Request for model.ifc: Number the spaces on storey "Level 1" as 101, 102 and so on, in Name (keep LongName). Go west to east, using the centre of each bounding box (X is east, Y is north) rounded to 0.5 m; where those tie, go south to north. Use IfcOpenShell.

First a look at what the model holds.

```python
import ifcopenshell
import ifcopenshell.util.element
import ifcopenshell.util.placement

model = ifcopenshell.open("model.ifc")
print(model.schema)
storey = next(s for s in model.by_type("IfcBuildingStorey") if s.Name == "Level 1")
spaces = [e for e in ifcopenshell.util.element.get_decomposition(storey) if e.is_a("IfcSpace")]
for e in sorted(spaces, key=lambda e: e.id()):
    origin = ifcopenshell.util.placement.get_local_placement(e.ObjectPlacement)[:3, 3]
    print(e.id(), e.Name, e.LongName, origin.round(2) + 0.0, sep=" | ")
```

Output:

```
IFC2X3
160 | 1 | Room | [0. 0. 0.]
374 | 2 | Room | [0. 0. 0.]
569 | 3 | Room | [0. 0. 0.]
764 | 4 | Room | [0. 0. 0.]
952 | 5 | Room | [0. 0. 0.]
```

```python
import ifcopenshell
import ifcopenshell.geom
import ifcopenshell.util.element
import ifcopenshell.util.shape

model = ifcopenshell.open("model.ifc")
settings = ifcopenshell.geom.settings()
settings.set("use-world-coords", True)


def centre(element):
    shape = ifcopenshell.geom.create_shape(settings, element)
    return ifcopenshell.util.shape.get_bbox_centroid(shape.geometry)


storey = next(s for s in model.by_type("IfcBuildingStorey") if s.Name == "Level 1")
spaces = [e for e in ifcopenshell.util.element.get_decomposition(storey) if e.is_a("IfcSpace")]

# Insertion points can sit at a corner or the storey origin, so sort by the geometry (in metres).
centres = {e: centre(e) for e in spaces}
spaces.sort(key=lambda e: (round(centres[e][0] / 0.5), centres[e][1]))

for i, e in enumerate(spaces, start=1):
    number = f"1{i:02d}"
    e.Name = number
    print(e.id(), number)

model.write("model_v2.ifc")
```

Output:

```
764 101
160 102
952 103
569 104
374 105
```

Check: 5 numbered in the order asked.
